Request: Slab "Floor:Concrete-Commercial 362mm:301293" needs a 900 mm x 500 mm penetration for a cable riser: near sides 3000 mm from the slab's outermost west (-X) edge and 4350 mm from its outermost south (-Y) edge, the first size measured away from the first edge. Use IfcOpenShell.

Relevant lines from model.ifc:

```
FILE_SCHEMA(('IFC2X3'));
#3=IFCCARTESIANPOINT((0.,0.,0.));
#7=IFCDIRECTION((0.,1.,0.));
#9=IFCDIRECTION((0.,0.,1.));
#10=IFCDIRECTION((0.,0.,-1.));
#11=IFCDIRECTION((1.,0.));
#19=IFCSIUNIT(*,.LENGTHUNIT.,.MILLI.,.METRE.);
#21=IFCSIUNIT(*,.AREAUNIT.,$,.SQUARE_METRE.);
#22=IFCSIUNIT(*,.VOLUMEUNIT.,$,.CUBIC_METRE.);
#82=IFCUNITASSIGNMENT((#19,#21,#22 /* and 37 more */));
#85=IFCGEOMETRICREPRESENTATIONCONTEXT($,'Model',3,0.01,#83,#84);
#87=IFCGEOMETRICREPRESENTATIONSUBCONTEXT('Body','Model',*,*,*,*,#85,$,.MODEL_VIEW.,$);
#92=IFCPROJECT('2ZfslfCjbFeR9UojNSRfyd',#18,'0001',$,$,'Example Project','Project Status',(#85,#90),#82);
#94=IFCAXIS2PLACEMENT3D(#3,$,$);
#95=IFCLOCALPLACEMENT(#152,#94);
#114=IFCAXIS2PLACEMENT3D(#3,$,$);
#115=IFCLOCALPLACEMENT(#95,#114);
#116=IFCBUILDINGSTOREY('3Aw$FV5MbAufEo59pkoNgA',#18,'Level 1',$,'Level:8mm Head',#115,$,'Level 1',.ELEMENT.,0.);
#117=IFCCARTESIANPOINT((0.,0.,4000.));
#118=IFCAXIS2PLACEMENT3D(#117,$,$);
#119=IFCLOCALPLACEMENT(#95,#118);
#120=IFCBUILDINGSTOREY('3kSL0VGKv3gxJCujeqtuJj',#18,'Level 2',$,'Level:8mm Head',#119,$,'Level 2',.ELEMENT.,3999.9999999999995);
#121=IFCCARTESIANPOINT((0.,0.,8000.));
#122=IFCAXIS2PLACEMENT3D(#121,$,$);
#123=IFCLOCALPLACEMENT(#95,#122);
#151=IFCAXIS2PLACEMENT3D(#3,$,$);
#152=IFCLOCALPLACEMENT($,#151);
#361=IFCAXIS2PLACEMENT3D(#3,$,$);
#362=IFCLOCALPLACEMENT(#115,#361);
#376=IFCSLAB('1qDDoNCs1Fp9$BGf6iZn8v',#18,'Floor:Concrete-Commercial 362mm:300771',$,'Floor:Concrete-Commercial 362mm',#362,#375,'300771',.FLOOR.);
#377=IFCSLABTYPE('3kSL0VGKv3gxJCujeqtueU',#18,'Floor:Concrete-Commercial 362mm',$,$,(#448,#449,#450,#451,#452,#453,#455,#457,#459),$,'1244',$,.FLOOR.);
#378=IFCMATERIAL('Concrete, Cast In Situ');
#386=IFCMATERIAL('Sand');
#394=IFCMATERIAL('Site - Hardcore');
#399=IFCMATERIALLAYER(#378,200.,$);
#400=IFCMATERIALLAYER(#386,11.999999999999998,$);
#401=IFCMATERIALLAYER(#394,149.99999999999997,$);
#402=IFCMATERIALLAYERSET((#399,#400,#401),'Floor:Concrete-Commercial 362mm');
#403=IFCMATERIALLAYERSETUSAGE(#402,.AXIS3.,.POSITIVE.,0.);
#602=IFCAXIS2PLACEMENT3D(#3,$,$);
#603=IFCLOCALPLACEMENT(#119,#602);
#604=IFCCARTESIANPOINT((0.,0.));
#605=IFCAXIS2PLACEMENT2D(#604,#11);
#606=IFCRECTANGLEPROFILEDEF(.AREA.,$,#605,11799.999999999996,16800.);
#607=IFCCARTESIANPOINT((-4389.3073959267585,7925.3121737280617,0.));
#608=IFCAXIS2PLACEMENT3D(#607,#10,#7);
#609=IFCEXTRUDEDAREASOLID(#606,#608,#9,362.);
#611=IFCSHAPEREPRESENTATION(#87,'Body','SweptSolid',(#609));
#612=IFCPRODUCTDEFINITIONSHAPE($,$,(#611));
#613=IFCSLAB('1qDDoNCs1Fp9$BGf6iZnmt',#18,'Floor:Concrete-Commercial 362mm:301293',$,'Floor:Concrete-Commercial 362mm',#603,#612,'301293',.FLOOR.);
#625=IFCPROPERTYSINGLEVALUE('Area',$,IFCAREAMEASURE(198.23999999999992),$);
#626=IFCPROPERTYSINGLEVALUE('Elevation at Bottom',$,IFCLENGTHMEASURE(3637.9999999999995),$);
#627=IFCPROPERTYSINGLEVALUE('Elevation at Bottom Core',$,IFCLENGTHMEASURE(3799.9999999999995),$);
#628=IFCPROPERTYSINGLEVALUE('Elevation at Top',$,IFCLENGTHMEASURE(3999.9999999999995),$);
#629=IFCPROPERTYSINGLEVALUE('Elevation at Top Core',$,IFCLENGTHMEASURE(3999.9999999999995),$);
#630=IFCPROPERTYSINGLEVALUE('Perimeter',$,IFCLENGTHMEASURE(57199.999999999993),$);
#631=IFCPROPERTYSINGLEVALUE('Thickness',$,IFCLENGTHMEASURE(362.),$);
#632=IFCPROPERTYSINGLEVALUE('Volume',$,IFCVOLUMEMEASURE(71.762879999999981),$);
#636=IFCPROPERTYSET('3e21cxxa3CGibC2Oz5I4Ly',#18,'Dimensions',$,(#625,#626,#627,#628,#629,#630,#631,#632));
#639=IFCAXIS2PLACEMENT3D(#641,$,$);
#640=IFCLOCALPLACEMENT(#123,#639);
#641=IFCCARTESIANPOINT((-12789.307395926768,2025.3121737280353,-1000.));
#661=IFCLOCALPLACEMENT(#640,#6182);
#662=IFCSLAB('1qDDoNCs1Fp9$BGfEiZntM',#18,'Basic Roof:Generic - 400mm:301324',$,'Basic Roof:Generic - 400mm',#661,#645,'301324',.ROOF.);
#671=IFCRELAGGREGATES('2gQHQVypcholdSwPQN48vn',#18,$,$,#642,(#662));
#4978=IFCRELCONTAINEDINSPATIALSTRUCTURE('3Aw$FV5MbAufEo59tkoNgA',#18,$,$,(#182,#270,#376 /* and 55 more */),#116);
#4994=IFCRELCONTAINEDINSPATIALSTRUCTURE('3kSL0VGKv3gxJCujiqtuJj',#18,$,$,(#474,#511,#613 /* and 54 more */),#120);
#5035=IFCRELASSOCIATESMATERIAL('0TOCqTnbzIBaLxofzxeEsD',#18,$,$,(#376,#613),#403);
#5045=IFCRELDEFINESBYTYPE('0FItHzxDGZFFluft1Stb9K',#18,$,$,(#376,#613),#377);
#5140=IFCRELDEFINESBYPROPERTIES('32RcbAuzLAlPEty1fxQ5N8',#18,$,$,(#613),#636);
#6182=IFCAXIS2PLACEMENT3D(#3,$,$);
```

```python
import numpy as np
import ifcopenshell
import ifcopenshell.api.feature
import ifcopenshell.api.geometry
import ifcopenshell.api.pset
import ifcopenshell.api.root
import ifcopenshell.geom
import ifcopenshell.util.element
import ifcopenshell.util.placement
import ifcopenshell.util.representation
import ifcopenshell.util.shape
import ifcopenshell.util.unit

model = ifcopenshell.open("model.ifc")
unit_scale = ifcopenshell.util.unit.calculate_unit_scale(model)
area_scale = ifcopenshell.util.unit.calculate_unit_scale(model, "AREAUNIT")
volume_scale = ifcopenshell.util.unit.calculate_unit_scale(model, "VOLUMEUNIT")
settings = ifcopenshell.geom.settings()


def volume(element):
    """Net volume in cubic metres, openings subtracted."""
    shape = ifcopenshell.geom.create_shape(settings, element)
    return ifcopenshell.util.shape.get_volume(shape.geometry)


slab = model.by_id(613)
before = volume(slab)

# Extent in the slab's own axes, in metres. The edges named are its -X and -Y sides.
slab_shape = ifcopenshell.geom.create_shape(settings, slab)
vertices = ifcopenshell.util.shape.get_vertices(slab_shape.geometry)
x_min, y_min, bottom = vertices.min(axis=0)
top = vertices[:, 2].max()

opening = ifcopenshell.api.root.create_entity(model, ifc_class="IfcOpeningElement", name="Cable riser opening")
context = ifcopenshell.util.representation.get_context(model, "Model", "Body", "MODEL_VIEW")
width, depth = 0.9, 0.5
outline = [(0.0, 0.0), (width, 0.0), (width, depth), (0.0, depth), (0.0, 0.0)]
# Overshoot both faces by 50 mm so the cut is clean.
shape = ifcopenshell.api.geometry.add_slab_representation(
    model, context=context, depth=top - bottom + 0.1, polyline=outline
)
ifcopenshell.api.geometry.assign_representation(model, product=opening, representation=shape)

matrix = ifcopenshell.util.placement.get_local_placement(slab.ObjectPlacement)
matrix[:, 3] = matrix @ np.append(np.array([x_min + 3, y_min + 4.35, bottom - 0.05]) / unit_scale, 1.0)
ifcopenshell.api.geometry.edit_object_placement(model, product=opening, matrix=matrix, is_si=False)
ifcopenshell.api.feature.add_feature(model, feature=opening, element=slab)

after = volume(slab)

# Update the slab's stored quantities.
pset = model.by_id(ifcopenshell.util.element.get_pset(slab, "Dimensions", should_inherit=False)["id"])
ifcopenshell.api.pset.edit_pset(model, pset=pset, properties={
    "Area": model.create_entity("IfcAreaMeasure", after / (top - bottom) / area_scale),
    "Volume": model.create_entity("IfcVolumeMeasure", after / volume_scale),
})

print(f"slab volume {before:.3f} -> {after:.3f} m3")

model.write("model_v2.ifc")
```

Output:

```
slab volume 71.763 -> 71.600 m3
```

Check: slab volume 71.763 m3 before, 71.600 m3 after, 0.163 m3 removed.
